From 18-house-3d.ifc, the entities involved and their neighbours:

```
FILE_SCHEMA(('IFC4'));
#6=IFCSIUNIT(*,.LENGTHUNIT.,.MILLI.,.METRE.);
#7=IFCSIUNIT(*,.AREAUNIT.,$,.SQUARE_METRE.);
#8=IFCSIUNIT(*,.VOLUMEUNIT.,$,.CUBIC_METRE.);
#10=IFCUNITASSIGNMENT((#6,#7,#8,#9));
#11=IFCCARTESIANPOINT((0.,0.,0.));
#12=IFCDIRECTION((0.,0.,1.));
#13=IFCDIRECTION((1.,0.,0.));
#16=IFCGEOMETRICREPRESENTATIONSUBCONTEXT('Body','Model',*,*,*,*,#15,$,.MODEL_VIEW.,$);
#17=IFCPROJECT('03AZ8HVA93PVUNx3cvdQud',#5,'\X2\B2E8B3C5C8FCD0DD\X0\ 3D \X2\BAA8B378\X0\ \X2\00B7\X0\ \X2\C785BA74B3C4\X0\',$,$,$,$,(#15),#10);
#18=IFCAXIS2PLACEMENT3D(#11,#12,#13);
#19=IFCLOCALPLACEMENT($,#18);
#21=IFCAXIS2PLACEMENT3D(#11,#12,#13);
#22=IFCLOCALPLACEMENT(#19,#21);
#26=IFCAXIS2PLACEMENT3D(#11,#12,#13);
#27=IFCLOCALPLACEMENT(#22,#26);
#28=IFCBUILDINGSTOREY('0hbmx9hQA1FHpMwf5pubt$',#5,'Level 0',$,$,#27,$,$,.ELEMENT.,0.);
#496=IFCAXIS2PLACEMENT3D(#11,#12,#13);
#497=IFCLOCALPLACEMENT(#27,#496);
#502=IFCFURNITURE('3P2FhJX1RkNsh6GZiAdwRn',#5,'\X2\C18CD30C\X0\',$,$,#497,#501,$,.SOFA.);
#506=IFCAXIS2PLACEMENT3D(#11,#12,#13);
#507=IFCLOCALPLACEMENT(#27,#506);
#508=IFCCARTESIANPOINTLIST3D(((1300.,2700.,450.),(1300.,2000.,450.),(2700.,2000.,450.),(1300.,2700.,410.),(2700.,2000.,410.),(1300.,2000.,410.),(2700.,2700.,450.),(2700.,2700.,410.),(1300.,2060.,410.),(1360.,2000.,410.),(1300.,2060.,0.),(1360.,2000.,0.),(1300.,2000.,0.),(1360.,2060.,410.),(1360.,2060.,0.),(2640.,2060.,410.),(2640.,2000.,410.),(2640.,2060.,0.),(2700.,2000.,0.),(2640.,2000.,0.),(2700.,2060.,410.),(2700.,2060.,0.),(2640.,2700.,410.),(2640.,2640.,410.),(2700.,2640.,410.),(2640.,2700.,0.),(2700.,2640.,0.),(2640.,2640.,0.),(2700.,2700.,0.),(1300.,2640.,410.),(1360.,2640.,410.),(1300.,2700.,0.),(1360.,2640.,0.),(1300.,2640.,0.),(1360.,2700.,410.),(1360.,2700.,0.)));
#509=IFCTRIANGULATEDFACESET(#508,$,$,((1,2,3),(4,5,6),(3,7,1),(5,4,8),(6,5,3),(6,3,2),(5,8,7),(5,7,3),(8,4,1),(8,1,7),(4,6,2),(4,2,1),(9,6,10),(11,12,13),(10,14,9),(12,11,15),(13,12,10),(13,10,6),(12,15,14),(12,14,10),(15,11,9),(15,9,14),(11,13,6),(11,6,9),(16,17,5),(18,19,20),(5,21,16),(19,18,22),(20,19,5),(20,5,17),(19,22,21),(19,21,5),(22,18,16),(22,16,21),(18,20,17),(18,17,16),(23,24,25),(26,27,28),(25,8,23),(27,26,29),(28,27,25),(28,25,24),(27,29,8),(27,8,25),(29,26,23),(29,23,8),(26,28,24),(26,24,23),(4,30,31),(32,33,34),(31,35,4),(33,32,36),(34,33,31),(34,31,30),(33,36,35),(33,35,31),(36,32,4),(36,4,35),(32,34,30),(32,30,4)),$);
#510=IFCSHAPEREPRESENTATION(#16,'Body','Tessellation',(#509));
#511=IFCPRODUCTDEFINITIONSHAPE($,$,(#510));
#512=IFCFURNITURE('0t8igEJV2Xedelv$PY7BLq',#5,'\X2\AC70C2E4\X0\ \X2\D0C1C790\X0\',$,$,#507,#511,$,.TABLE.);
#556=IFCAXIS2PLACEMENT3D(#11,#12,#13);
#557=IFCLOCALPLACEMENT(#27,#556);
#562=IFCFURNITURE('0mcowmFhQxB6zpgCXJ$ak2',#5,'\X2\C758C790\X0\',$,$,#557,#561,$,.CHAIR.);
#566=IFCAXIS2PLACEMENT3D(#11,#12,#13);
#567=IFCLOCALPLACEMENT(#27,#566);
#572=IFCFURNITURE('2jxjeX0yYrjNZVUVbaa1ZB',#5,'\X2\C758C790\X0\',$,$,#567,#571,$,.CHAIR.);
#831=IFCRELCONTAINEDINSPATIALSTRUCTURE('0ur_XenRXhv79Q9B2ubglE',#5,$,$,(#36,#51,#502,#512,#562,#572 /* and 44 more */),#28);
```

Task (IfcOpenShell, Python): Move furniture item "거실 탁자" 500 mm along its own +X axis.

```python
import ifcopenshell
import ifcopenshell.api.geometry
import ifcopenshell.util.placement

model = ifcopenshell.open("18-house-3d.ifc")

item = model.by_id(512)
matrix = ifcopenshell.util.placement.get_local_placement(item.ObjectPlacement)
matrix[:3, 3] += matrix[:3, 0] * 500.0
ifcopenshell.api.geometry.edit_object_placement(model, product=item, matrix=matrix, is_si=False)

print(ifcopenshell.util.placement.get_local_placement(item.ObjectPlacement).round(3) + 0.0)

model.write("18-house-3d_v2.ifc")
```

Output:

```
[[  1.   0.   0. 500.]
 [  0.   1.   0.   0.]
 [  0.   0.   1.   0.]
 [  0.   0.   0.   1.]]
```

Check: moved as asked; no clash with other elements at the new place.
